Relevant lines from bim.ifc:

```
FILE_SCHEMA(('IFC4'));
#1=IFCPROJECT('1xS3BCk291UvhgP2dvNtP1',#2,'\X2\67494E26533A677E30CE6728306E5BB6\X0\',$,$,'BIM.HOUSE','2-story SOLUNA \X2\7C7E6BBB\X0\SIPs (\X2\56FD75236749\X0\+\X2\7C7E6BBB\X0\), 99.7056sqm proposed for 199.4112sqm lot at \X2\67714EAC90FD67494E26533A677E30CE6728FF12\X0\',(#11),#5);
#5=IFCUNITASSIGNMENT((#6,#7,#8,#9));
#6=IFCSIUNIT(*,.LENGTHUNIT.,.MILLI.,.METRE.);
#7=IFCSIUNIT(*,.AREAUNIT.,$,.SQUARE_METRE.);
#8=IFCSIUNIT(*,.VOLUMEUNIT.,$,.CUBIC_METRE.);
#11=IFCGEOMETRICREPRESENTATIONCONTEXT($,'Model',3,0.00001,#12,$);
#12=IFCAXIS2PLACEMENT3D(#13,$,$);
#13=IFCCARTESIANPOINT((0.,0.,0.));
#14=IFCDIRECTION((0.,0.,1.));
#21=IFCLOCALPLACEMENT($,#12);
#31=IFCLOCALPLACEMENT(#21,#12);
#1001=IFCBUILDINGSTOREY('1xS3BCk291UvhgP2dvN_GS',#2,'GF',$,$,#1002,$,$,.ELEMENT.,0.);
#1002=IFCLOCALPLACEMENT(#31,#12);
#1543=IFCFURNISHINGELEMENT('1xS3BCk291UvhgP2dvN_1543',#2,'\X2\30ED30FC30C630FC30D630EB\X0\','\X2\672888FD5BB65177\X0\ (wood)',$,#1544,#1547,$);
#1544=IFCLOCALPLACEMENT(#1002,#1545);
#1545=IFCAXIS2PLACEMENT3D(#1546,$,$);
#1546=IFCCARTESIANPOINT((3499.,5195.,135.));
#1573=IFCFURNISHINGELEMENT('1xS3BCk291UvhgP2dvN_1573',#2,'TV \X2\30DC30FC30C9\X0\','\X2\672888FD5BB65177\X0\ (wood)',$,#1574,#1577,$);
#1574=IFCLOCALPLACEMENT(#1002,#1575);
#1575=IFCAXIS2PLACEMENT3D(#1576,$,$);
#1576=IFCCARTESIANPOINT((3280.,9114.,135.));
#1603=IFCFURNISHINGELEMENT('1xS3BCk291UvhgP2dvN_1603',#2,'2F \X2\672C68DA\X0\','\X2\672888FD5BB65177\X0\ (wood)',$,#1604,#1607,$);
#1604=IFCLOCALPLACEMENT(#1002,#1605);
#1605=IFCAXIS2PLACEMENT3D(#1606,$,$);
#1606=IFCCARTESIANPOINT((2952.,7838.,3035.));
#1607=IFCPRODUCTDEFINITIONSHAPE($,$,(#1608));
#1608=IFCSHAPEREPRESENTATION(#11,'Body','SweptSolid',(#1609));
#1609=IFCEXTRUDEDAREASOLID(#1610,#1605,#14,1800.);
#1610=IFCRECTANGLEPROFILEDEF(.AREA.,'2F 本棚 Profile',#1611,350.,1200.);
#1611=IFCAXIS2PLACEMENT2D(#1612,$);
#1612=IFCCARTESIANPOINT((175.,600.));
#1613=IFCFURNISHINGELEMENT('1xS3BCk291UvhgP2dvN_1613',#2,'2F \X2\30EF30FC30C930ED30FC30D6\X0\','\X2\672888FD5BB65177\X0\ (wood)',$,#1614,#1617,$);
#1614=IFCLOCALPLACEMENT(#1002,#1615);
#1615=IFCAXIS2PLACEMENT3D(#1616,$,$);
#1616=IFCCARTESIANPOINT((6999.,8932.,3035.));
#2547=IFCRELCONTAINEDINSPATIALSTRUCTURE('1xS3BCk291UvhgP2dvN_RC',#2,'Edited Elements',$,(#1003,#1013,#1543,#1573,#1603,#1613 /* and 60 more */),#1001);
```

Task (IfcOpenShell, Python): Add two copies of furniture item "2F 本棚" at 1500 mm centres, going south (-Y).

```python
import numpy as np
import ifcopenshell
import ifcopenshell.api.geometry
import ifcopenshell.api.root
import ifcopenshell.util.element
import ifcopenshell.util.placement

model = ifcopenshell.open("bim.ifc")


def reuse_history(source, copy):
    """copy_class also copies each property set's owner history, people and application; keep the originals."""
    for rel in copy.IsDefinedBy:
        if rel.is_a("IfcRelDefinesByProperties") and (history := rel.RelatingPropertyDefinition.OwnerHistory):
            rel.RelatingPropertyDefinition.OwnerHistory = source.OwnerHistory
            ifcopenshell.util.element.remove_deep2(model, history)


source = model.by_guid("1xS3BCk291UvhgP2dvN_1603")
base = ifcopenshell.util.placement.get_local_placement(source.ObjectPlacement)
step = np.array([0.0, -1.0, 0.0]) * 1500.0

for i in range(1, 3):
    copy = ifcopenshell.api.root.copy_class(model, product=source)
    copy.Representation = ifcopenshell.util.element.copy_deep(
        model, source.Representation, exclude=["IfcGeometricRepresentationContext", "IfcRepresentationMap"]
    )
    reuse_history(source, copy)
    matrix = base.copy()
    matrix[:3, 3] += i * step
    print("added at", matrix[:3, 3].round(3) + 0.0)
    ifcopenshell.api.geometry.edit_object_placement(model, product=copy, matrix=matrix, is_si=False)

model.write("bim_v2.ifc")
```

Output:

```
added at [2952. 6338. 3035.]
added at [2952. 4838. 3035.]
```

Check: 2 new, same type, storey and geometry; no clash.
